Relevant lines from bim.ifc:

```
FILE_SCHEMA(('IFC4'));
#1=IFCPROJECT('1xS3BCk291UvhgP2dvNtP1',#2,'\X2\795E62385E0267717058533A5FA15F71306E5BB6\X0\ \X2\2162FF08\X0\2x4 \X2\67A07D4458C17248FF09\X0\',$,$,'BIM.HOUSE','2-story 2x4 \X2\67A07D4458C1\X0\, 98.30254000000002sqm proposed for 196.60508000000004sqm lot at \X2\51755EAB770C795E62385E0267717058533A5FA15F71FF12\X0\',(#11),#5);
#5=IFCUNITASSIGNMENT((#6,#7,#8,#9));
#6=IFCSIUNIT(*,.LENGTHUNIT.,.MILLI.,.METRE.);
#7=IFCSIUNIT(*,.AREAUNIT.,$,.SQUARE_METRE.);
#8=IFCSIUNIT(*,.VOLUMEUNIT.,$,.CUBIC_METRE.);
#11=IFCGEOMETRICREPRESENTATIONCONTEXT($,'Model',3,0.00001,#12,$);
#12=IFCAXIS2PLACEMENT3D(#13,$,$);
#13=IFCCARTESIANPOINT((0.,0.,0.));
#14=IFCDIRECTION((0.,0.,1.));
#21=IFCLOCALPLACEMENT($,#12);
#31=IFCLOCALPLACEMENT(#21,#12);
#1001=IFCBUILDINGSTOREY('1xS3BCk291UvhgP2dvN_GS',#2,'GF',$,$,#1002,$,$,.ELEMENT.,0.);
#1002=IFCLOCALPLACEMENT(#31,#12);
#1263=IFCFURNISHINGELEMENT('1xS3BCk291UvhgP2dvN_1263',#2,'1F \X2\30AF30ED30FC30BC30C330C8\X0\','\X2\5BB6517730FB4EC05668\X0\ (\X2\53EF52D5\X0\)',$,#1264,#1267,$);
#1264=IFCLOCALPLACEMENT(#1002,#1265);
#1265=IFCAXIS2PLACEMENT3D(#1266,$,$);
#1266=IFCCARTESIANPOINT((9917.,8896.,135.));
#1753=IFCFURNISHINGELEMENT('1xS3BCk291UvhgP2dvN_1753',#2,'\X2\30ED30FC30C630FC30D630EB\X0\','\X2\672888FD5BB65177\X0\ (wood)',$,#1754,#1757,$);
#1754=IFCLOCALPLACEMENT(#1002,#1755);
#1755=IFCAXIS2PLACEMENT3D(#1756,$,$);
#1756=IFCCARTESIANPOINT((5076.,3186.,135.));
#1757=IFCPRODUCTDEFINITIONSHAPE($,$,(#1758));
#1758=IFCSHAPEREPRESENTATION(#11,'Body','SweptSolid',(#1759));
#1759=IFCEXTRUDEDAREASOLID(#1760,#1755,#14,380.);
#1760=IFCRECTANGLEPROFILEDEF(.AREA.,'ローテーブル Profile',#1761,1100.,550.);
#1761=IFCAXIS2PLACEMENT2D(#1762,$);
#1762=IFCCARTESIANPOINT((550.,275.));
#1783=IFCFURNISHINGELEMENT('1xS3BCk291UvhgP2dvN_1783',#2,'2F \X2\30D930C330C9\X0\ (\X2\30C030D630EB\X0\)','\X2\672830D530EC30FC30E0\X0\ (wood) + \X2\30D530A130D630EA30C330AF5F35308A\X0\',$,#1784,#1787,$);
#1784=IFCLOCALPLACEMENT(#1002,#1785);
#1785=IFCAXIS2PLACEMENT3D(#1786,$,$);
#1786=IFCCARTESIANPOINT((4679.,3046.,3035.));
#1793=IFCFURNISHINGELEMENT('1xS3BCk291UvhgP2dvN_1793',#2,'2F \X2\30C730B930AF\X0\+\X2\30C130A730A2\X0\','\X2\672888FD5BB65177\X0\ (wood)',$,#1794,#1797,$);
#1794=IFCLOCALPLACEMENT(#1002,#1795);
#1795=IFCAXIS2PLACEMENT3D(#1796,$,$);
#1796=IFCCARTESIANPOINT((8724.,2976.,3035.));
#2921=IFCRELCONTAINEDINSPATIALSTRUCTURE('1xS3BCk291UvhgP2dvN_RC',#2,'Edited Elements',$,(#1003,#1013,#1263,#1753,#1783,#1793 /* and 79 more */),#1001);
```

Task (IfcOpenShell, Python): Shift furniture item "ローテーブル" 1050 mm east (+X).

```python
import ifcopenshell
import ifcopenshell.api.geometry
import ifcopenshell.util.placement

model = ifcopenshell.open("bim.ifc")

item = model.by_guid("1xS3BCk291UvhgP2dvN_1753")
matrix = ifcopenshell.util.placement.get_local_placement(item.ObjectPlacement)
matrix[0, 3] += 1050.0
ifcopenshell.api.geometry.edit_object_placement(model, product=item, matrix=matrix, is_si=False)

print(ifcopenshell.util.placement.get_local_placement(item.ObjectPlacement).round(3) + 0.0)

model.write("bim_rev.ifc")
```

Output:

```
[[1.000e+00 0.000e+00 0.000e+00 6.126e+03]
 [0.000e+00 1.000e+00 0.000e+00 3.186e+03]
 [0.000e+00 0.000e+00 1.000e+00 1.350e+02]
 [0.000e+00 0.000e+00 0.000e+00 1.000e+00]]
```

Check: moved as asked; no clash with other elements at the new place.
